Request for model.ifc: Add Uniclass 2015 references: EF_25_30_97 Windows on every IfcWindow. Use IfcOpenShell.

First a look at what the model holds.

```python
import ifcopenshell

model = ifcopenshell.open("model.ifc")
print(model.schema)
print("classifications:", [c.Name for c in model.by_type("IfcClassification")])
for ifc_class in ("IfcDoor", "IfcRoof", "IfcStair", "IfcWall", "IfcWindow"):
    print(ifc_class, len(model.by_type(ifc_class)))
```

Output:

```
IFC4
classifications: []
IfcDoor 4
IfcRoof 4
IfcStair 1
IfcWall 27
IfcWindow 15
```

```python
import ifcopenshell
import ifcopenshell.api.classification

model = ifcopenshell.open("model.ifc")

system = ifcopenshell.api.classification.add_classification(model, classification="Uniclass 2015")

codes = {
    "IfcWindow": ("EF_25_30_97", "Windows"),
}
for ifc_class, (code, name) in codes.items():
    products = model.by_type(ifc_class)
    ifcopenshell.api.classification.add_reference(
        model, products=products, classification=system, identification=code, name=name
    )
    print(code, len(products))

model.write("model-out.ifc")
```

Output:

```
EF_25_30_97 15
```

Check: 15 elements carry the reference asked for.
